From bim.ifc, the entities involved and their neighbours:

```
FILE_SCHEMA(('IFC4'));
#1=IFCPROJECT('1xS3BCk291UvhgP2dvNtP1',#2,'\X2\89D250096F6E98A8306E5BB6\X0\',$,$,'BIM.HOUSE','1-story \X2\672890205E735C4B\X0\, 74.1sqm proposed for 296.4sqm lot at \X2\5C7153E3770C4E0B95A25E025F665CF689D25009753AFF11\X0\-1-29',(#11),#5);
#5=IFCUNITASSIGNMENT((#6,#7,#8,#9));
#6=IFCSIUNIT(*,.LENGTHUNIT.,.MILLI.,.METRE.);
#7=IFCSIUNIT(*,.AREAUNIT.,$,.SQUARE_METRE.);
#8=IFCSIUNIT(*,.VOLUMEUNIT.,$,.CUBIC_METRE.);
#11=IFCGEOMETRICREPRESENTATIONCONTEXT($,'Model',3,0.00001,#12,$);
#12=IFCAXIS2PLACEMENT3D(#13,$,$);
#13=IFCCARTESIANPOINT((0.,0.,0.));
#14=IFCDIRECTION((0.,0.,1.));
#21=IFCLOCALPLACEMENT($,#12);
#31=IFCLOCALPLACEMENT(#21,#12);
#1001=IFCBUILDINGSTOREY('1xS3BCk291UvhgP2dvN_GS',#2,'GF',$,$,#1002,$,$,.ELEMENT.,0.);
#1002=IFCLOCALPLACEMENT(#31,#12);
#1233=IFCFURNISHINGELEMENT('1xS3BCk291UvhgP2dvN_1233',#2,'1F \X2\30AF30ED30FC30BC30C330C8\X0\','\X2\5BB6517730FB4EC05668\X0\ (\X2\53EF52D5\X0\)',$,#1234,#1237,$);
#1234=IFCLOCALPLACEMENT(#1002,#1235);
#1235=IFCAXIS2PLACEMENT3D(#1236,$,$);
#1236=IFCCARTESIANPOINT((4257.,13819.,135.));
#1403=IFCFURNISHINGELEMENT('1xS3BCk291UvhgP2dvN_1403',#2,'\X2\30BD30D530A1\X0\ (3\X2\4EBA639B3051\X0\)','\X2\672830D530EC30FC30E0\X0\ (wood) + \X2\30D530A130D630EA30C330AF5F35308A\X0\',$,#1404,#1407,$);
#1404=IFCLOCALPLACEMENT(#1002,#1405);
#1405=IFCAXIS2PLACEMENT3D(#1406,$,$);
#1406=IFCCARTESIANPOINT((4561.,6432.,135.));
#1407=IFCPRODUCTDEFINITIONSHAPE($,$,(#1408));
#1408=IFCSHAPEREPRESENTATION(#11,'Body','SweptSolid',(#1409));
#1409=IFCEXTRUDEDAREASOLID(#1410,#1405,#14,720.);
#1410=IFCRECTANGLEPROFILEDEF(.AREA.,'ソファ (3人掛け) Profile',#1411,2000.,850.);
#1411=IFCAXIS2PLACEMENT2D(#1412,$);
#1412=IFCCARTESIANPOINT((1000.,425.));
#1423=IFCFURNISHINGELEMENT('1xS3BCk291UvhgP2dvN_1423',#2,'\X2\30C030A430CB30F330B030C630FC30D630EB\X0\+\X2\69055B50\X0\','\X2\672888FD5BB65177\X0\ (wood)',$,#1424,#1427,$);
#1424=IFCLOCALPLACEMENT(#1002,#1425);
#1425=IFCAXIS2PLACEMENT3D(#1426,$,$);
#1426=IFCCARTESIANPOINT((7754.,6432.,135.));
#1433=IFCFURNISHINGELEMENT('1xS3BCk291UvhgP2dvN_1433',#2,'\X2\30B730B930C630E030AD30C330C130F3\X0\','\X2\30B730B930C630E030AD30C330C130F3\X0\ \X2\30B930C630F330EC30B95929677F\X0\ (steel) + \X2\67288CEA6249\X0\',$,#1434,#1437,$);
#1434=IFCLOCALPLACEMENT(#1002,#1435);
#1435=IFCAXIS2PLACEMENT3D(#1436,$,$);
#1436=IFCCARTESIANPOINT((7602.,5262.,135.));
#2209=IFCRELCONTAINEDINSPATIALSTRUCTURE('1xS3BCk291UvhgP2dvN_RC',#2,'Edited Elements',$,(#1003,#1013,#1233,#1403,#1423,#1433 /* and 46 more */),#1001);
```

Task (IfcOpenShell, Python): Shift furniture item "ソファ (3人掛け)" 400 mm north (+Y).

```python
import ifcopenshell
import ifcopenshell.api.geometry
import ifcopenshell.util.placement
import ifcopenshell.util.unit

model = ifcopenshell.open("bim.ifc")
unit_scale = ifcopenshell.util.unit.calculate_unit_scale(model)

item = model.by_guid("1xS3BCk291UvhgP2dvN_1403")
matrix = ifcopenshell.util.placement.get_local_placement(item.ObjectPlacement)
matrix[1, 3] += 0.4 / unit_scale
ifcopenshell.api.geometry.edit_object_placement(model, product=item, matrix=matrix, is_si=False)

print(ifcopenshell.util.placement.get_local_placement(item.ObjectPlacement).round(3) + 0.0)

model.write("bim_edited.ifc")
```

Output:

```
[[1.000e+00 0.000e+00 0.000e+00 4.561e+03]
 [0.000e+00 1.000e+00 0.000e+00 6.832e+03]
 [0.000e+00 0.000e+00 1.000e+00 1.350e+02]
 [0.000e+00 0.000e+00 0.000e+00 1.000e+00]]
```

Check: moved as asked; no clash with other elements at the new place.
